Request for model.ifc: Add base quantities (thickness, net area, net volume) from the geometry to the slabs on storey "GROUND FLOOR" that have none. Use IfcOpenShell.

First a look at what the model holds.

```python
import ifcopenshell
import ifcopenshell.util.element
import ifcopenshell.util.unit

model = ifcopenshell.open("model.ifc")
print(model.schema)
for unit_type in ("LENGTHUNIT", "AREAUNIT", "VOLUMEUNIT"):
    print(unit_type, ifcopenshell.util.unit.calculate_unit_scale(model, unit_type))
storey = next(s for s in model.by_type("IfcBuildingStorey") if s.Name == "GROUND FLOOR")
slabs = [e for e in ifcopenshell.util.element.get_decomposition(storey) if e.is_a("IfcSlab")]
for e in sorted(slabs, key=lambda e: e.id()):
    print(e.id(), e.is_a(), e.Name, list(ifcopenshell.util.element.get_psets(e, qtos_only=True)), sep=" | ")
```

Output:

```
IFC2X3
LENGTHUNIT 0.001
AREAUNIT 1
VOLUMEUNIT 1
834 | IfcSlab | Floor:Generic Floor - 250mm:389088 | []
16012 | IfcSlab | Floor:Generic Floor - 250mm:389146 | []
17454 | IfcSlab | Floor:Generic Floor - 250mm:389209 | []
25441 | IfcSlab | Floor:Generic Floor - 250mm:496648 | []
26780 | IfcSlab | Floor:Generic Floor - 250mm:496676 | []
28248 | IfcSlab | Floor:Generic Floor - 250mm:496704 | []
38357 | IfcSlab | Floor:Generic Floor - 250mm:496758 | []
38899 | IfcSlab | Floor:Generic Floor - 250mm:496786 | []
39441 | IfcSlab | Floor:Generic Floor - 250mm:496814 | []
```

```python
import ifcopenshell
import ifcopenshell.api.pset
import ifcopenshell.geom
import ifcopenshell.util.element
import ifcopenshell.util.shape
import ifcopenshell.util.unit

model = ifcopenshell.open("model.ifc")
unit_scale = ifcopenshell.util.unit.calculate_unit_scale(model)
area_scale = ifcopenshell.util.unit.calculate_unit_scale(model, "AREAUNIT")
volume_scale = ifcopenshell.util.unit.calculate_unit_scale(model, "VOLUMEUNIT")
settings = ifcopenshell.geom.settings()

storey = next(s for s in model.by_type("IfcBuildingStorey") if s.Name == "GROUND FLOOR")
slabs = [e for e in ifcopenshell.util.element.get_decomposition(storey) if e.is_a("IfcSlab")]

for e in sorted(slabs, key=lambda e: e.id()):
    if ifcopenshell.util.element.get_psets(e, qtos_only=True, should_inherit=False):
        continue
    # Geometry comes back in metres, in the element's own axes.
    shape = ifcopenshell.geom.create_shape(settings, e)
    values = {
        "Width": ifcopenshell.util.shape.get_z(shape.geometry) / unit_scale,
        "NetArea": ifcopenshell.util.shape.get_footprint_area(shape.geometry) / area_scale,
        "NetVolume": ifcopenshell.util.shape.get_volume(shape.geometry) / volume_scale,
    }
    qto = ifcopenshell.api.pset.add_qto(model, product=e, name="BaseQuantities")
    ifcopenshell.api.pset.edit_qto(model, qto=qto, properties=values)
    print(e.id(), {k: round(v, 3) for k, v in values.items()})

model.write("model_edited.ifc")
```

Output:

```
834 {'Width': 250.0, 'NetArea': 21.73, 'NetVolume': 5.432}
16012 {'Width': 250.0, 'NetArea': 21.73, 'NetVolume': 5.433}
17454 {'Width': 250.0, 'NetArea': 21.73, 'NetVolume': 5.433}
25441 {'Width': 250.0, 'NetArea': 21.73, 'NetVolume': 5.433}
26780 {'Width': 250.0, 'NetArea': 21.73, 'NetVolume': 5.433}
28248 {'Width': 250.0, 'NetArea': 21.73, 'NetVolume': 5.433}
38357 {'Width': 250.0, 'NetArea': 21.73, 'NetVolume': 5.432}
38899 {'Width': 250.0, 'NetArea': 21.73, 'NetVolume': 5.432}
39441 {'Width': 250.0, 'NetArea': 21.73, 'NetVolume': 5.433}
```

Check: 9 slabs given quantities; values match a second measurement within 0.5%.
